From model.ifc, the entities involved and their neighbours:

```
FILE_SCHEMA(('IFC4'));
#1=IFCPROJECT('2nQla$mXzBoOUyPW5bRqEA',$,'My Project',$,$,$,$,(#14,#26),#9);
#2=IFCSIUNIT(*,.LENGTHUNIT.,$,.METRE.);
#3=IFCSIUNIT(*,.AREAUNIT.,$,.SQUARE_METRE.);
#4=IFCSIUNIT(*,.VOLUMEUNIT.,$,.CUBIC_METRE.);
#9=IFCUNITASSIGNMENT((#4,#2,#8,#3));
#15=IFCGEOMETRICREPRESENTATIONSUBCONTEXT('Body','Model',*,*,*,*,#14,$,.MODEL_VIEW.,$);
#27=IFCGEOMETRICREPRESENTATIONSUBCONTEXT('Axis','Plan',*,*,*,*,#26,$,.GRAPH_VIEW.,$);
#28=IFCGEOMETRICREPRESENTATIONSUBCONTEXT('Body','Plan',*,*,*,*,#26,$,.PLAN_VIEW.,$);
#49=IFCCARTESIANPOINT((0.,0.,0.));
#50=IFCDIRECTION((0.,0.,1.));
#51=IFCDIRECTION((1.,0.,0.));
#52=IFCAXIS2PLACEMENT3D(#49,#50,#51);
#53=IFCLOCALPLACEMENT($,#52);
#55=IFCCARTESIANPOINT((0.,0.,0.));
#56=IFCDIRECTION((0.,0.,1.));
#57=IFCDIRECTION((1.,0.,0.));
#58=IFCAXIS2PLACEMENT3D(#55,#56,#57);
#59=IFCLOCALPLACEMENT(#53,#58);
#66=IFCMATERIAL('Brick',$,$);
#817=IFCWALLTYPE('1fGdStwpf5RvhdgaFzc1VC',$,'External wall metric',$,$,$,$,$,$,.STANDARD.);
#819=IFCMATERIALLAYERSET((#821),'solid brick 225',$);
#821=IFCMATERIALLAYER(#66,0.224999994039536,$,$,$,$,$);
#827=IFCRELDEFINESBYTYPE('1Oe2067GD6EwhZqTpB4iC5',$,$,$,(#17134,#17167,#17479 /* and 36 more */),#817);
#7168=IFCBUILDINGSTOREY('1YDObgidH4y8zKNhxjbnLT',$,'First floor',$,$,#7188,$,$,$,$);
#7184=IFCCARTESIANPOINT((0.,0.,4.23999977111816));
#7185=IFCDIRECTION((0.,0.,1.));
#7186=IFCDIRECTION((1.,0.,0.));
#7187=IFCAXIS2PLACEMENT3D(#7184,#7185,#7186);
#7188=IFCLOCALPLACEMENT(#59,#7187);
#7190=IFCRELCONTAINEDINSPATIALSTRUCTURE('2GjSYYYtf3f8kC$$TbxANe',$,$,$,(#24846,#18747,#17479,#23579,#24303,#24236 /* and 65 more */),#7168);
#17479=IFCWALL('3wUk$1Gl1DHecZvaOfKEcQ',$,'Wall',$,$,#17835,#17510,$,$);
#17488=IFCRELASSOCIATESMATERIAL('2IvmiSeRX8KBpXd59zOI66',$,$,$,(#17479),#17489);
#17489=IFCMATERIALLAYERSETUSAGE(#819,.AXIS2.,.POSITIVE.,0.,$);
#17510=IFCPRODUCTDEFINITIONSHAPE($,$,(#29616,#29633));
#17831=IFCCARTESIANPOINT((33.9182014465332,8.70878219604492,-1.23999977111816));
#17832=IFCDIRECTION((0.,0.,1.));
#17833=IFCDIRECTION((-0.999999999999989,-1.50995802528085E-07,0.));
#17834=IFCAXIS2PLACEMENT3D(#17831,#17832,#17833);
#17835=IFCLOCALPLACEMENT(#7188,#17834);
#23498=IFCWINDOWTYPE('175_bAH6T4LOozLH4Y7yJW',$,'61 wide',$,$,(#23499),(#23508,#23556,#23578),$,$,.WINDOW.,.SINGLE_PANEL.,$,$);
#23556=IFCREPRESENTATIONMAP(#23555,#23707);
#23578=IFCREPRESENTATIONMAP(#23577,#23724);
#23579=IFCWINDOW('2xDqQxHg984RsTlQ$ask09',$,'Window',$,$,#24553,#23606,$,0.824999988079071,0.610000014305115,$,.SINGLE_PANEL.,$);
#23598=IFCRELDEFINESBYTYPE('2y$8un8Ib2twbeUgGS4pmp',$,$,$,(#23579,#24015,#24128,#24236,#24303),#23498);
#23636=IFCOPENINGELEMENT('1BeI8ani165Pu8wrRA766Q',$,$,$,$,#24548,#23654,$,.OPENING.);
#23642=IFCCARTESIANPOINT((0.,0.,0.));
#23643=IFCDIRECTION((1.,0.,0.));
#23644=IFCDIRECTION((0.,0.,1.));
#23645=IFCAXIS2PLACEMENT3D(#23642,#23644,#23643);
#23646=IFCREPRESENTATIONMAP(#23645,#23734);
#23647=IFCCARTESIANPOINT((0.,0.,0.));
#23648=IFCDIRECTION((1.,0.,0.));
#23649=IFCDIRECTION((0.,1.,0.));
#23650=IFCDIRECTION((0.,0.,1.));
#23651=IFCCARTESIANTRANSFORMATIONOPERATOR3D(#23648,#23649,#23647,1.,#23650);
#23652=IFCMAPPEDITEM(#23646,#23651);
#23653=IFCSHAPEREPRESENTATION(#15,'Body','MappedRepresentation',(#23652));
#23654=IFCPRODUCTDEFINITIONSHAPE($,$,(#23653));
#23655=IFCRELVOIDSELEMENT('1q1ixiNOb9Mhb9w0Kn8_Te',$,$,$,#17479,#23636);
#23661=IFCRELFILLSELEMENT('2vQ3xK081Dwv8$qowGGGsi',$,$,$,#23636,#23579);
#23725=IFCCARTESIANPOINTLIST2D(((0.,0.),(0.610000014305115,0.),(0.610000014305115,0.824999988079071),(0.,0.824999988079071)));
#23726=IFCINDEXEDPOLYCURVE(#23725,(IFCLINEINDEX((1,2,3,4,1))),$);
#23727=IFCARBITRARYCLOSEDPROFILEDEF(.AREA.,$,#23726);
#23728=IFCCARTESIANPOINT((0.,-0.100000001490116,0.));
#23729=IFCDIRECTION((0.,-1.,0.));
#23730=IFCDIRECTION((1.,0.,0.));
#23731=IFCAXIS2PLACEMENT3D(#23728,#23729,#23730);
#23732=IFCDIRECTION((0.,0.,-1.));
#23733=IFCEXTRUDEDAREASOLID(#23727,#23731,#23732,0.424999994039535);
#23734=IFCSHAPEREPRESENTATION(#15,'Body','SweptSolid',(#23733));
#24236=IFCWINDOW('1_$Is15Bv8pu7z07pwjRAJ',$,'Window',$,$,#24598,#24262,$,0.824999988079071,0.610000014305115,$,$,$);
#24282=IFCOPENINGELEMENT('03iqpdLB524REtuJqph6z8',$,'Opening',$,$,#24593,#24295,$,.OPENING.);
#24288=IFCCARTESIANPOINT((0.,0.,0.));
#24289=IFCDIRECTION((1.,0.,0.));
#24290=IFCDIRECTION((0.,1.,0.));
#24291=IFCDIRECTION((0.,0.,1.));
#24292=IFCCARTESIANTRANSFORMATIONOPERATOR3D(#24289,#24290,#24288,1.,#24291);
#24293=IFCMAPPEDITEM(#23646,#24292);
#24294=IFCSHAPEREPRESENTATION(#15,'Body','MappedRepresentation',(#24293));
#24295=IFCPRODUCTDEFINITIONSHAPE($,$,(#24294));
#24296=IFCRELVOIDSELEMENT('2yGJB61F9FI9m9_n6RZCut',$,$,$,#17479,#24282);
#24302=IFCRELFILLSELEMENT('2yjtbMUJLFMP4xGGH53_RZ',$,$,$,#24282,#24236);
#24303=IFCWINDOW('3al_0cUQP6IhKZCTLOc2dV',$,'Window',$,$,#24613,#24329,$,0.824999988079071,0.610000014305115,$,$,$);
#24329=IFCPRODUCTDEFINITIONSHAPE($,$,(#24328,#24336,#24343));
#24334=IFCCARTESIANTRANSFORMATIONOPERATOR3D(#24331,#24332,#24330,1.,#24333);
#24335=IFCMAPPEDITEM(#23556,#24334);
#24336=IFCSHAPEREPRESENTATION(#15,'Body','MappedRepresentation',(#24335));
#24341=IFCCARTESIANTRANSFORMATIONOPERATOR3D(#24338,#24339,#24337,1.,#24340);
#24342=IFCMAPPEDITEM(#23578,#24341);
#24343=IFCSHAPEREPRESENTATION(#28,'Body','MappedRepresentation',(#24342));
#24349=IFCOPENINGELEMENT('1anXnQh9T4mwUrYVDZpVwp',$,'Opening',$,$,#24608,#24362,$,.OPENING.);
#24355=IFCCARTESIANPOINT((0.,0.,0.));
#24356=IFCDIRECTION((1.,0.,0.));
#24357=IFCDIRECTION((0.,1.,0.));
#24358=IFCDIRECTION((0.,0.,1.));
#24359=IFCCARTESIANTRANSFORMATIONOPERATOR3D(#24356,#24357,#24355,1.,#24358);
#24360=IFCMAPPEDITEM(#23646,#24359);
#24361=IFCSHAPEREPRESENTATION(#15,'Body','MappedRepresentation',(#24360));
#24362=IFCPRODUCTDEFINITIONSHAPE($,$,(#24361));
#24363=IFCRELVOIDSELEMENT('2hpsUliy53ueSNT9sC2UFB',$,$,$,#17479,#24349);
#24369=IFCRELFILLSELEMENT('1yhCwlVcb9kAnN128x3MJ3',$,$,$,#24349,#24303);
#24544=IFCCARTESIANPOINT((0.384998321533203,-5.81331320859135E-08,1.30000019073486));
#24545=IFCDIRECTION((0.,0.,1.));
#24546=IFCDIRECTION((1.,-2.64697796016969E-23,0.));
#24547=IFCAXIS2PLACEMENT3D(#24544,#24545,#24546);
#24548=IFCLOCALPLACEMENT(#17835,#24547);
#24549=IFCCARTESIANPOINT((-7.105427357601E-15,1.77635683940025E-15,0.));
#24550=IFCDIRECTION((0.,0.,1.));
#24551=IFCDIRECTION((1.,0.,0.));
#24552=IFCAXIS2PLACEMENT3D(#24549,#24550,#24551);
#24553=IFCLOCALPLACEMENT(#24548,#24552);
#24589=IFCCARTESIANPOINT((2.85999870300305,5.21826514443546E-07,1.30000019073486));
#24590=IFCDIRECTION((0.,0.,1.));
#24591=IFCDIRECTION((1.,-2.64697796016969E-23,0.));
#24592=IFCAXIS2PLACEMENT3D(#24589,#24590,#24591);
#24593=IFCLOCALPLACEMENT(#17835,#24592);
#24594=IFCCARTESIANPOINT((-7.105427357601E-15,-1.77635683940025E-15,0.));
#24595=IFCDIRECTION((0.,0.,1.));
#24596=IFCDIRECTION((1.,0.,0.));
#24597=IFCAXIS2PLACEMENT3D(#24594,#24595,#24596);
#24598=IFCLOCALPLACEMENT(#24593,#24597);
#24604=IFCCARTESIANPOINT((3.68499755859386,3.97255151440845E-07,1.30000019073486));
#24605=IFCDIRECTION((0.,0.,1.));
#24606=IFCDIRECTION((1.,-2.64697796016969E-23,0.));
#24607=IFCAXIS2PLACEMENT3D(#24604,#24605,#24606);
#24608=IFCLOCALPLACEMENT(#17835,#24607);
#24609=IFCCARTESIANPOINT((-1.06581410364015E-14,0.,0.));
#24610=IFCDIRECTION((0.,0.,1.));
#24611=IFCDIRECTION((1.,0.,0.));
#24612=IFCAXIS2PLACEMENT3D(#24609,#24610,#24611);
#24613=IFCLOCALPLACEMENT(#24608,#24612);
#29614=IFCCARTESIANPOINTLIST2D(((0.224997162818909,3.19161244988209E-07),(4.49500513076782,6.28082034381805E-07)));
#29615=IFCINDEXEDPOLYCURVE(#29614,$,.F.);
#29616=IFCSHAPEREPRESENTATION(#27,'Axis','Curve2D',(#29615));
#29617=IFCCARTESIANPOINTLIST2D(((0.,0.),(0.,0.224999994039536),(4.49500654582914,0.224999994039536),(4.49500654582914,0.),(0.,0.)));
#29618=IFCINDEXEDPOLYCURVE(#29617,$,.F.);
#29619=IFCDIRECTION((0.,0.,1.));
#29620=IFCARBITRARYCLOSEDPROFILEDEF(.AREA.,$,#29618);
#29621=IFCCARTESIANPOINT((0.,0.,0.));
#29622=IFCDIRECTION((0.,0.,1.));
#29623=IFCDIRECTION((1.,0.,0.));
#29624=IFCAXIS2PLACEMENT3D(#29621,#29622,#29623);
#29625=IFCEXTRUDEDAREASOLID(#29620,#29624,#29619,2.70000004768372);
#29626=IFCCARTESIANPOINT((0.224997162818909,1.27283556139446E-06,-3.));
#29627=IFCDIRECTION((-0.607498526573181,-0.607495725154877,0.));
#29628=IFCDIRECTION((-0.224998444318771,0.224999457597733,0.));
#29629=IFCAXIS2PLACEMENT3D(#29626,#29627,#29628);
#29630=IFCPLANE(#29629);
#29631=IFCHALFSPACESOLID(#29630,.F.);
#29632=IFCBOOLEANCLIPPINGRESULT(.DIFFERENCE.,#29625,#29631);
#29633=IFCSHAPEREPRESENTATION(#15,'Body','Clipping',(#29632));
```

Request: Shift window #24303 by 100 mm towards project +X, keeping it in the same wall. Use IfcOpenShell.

```python
import ifcopenshell
import ifcopenshell.api.geometry
import ifcopenshell.util.placement

model = ifcopenshell.open("model.ifc")

window = model.by_guid("3al_0cUQP6IhKZCTLOc2dV")
opening = window.FillsVoids[0].RelatingOpeningElement
wall = opening.VoidsElements[0].RelatingBuildingElement

wall_matrix = ifcopenshell.util.placement.get_local_placement(wall.ObjectPlacement)
shift = wall_matrix[:3, 0] * -0.1
before = ifcopenshell.util.placement.get_local_placement(window.ObjectPlacement)[:3, 3].copy()

# The window is placed relative to its opening, so it follows when the opening moves.
matrix = ifcopenshell.util.placement.get_local_placement(opening.ObjectPlacement)
matrix[:3, 3] += shift
ifcopenshell.api.geometry.edit_object_placement(
    model, product=opening, matrix=matrix, is_si=False, should_transform_children=True
)

after = ifcopenshell.util.placement.get_local_placement(window.ObjectPlacement)[:3, 3]
print("window moved by", (after - before).round(3) + 0.0)

model.write("model_updated.ifc")
```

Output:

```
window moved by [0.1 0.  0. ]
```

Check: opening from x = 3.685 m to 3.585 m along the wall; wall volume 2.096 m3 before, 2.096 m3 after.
